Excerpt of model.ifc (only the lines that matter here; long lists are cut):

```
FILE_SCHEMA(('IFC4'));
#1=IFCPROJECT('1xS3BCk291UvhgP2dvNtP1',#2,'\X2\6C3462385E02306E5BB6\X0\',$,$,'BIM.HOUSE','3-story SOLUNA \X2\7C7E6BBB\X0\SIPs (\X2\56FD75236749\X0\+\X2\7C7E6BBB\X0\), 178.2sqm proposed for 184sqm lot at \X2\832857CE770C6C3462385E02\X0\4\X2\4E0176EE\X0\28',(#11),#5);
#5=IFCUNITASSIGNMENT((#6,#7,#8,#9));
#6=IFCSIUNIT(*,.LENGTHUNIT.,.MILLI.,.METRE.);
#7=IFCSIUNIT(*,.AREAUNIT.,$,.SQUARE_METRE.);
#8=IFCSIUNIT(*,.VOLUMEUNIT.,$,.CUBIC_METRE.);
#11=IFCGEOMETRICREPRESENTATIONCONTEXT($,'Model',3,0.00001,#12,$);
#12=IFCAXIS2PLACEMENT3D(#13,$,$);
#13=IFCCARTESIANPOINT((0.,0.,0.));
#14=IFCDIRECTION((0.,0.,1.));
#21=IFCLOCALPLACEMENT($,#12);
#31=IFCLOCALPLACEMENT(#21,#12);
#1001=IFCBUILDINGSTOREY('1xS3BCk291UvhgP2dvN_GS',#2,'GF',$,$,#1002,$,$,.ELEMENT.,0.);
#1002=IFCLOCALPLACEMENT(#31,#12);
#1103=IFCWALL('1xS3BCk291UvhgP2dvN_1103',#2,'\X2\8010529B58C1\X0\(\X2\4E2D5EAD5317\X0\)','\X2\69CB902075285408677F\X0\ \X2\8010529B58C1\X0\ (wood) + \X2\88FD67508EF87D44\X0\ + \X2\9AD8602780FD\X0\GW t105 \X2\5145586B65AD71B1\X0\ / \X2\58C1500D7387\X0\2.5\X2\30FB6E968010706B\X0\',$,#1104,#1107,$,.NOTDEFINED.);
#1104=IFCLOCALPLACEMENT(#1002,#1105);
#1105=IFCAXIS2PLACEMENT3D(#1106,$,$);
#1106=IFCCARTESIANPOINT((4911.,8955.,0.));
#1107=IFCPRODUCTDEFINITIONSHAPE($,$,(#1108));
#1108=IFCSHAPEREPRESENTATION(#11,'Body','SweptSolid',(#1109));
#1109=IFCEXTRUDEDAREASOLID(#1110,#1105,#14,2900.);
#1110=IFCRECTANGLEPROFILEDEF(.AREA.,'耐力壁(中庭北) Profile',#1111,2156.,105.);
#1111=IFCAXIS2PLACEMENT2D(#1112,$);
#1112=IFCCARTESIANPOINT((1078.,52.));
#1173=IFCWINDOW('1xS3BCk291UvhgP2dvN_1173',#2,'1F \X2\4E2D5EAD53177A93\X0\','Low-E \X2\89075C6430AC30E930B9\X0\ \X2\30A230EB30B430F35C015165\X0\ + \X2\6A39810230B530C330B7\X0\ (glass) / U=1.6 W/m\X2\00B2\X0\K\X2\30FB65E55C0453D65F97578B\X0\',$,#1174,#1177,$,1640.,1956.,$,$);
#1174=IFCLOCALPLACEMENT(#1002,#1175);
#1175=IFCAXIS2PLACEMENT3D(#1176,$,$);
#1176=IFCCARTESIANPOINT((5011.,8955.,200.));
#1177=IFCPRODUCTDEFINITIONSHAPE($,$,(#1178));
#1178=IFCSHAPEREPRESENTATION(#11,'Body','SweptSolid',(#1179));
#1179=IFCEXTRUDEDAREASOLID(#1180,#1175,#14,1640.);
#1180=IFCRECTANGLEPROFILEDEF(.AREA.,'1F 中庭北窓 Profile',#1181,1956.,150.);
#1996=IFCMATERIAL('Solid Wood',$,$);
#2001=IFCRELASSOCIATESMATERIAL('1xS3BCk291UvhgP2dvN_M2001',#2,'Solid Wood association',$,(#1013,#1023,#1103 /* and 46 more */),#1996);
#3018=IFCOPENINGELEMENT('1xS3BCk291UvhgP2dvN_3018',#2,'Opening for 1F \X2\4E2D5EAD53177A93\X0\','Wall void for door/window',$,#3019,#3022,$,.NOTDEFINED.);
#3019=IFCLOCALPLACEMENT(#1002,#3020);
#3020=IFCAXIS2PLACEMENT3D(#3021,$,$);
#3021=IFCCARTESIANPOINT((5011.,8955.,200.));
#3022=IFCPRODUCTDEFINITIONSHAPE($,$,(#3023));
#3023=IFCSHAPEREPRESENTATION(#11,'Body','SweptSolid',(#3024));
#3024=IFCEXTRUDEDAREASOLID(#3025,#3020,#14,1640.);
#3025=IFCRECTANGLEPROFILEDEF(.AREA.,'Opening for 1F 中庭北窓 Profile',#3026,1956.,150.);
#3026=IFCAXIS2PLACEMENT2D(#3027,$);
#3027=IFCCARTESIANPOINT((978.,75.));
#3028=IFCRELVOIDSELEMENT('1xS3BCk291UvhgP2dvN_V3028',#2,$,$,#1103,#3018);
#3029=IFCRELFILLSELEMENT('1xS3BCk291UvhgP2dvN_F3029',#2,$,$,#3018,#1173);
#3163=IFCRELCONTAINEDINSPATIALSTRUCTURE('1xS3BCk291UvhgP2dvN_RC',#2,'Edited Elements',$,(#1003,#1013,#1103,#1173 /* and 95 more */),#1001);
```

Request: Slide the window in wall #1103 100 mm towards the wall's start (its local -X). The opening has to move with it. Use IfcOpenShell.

```python
import ifcopenshell
import ifcopenshell.api.geometry
import ifcopenshell.util.placement

model = ifcopenshell.open("model.ifc")

window = model.by_id(1173)
opening = window.FillsVoids[0].RelatingOpeningElement
wall = opening.VoidsElements[0].RelatingBuildingElement

wall_matrix = ifcopenshell.util.placement.get_local_placement(wall.ObjectPlacement)
shift = wall_matrix[:3, 0] * -100.0
before = ifcopenshell.util.placement.get_local_placement(window.ObjectPlacement)[:3, 3].copy()

# The window is not placed relative to its opening, so move both.
for product in (opening, window):
    matrix = ifcopenshell.util.placement.get_local_placement(product.ObjectPlacement)
    matrix[:3, 3] += shift
    ifcopenshell.api.geometry.edit_object_placement(model, product=product, matrix=matrix, is_si=False)

after = ifcopenshell.util.placement.get_local_placement(window.ObjectPlacement)[:3, 3]
print("window moved by", (after - before).round(3) + 0.0)

model.write("model_rev.ifc")
```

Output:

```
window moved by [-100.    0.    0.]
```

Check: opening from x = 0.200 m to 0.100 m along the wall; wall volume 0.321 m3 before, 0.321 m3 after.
